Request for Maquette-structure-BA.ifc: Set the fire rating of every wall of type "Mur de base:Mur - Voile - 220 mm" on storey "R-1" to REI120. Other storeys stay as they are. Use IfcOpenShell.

First a look at what the model holds.

```python
import ifcopenshell
import ifcopenshell.util.element

model = ifcopenshell.open("Maquette-structure-BA.ifc")
print(model.schema)
storey = next(s for s in model.by_type("IfcBuildingStorey") if s.Name == "R-1")
walls = [e for e in ifcopenshell.util.element.get_decomposition(storey) if e.is_a("IfcWall")]
seen = {}
for e in walls:
    element_type = ifcopenshell.util.element.get_type(e)
    key = (element_type.Name if element_type != e and element_type else None, ifcopenshell.util.element.get_pset(e, "Pset_WallCommon", "FireRating"))
    seen[key] = seen.get(key, 0) + 1
for (name, value), count in sorted(seen.items(), key=str):
    print(count, "x", name, "|", value)
```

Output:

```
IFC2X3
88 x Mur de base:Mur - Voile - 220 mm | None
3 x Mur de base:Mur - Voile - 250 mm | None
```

```python
import ifcopenshell
import ifcopenshell.api.pset
import ifcopenshell.util.element

model = ifcopenshell.open("Maquette-structure-BA.ifc")

storey = next(s for s in model.by_type("IfcBuildingStorey") if s.Name == "R-1")
walls = [e for e in ifcopenshell.util.element.get_decomposition(storey) if e.is_a("IfcWall")]

count = 0
for e in walls:
    element_type = ifcopenshell.util.element.get_type(e)
    if element_type in (None, e) or element_type.Name != "Mur de base:Mur - Voile - 220 mm":
        continue
    # add_pset returns the element's existing set when there is one.
    pset = ifcopenshell.api.pset.add_pset(model, product=e, name="Pset_WallCommon")
    ifcopenshell.api.pset.edit_pset(model, pset=pset, properties={"FireRating": "REI120"})
    count += 1

print(count, "walls updated")

model.write("Maquette-structure-BA_rev.ifc")
```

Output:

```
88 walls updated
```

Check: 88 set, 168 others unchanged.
